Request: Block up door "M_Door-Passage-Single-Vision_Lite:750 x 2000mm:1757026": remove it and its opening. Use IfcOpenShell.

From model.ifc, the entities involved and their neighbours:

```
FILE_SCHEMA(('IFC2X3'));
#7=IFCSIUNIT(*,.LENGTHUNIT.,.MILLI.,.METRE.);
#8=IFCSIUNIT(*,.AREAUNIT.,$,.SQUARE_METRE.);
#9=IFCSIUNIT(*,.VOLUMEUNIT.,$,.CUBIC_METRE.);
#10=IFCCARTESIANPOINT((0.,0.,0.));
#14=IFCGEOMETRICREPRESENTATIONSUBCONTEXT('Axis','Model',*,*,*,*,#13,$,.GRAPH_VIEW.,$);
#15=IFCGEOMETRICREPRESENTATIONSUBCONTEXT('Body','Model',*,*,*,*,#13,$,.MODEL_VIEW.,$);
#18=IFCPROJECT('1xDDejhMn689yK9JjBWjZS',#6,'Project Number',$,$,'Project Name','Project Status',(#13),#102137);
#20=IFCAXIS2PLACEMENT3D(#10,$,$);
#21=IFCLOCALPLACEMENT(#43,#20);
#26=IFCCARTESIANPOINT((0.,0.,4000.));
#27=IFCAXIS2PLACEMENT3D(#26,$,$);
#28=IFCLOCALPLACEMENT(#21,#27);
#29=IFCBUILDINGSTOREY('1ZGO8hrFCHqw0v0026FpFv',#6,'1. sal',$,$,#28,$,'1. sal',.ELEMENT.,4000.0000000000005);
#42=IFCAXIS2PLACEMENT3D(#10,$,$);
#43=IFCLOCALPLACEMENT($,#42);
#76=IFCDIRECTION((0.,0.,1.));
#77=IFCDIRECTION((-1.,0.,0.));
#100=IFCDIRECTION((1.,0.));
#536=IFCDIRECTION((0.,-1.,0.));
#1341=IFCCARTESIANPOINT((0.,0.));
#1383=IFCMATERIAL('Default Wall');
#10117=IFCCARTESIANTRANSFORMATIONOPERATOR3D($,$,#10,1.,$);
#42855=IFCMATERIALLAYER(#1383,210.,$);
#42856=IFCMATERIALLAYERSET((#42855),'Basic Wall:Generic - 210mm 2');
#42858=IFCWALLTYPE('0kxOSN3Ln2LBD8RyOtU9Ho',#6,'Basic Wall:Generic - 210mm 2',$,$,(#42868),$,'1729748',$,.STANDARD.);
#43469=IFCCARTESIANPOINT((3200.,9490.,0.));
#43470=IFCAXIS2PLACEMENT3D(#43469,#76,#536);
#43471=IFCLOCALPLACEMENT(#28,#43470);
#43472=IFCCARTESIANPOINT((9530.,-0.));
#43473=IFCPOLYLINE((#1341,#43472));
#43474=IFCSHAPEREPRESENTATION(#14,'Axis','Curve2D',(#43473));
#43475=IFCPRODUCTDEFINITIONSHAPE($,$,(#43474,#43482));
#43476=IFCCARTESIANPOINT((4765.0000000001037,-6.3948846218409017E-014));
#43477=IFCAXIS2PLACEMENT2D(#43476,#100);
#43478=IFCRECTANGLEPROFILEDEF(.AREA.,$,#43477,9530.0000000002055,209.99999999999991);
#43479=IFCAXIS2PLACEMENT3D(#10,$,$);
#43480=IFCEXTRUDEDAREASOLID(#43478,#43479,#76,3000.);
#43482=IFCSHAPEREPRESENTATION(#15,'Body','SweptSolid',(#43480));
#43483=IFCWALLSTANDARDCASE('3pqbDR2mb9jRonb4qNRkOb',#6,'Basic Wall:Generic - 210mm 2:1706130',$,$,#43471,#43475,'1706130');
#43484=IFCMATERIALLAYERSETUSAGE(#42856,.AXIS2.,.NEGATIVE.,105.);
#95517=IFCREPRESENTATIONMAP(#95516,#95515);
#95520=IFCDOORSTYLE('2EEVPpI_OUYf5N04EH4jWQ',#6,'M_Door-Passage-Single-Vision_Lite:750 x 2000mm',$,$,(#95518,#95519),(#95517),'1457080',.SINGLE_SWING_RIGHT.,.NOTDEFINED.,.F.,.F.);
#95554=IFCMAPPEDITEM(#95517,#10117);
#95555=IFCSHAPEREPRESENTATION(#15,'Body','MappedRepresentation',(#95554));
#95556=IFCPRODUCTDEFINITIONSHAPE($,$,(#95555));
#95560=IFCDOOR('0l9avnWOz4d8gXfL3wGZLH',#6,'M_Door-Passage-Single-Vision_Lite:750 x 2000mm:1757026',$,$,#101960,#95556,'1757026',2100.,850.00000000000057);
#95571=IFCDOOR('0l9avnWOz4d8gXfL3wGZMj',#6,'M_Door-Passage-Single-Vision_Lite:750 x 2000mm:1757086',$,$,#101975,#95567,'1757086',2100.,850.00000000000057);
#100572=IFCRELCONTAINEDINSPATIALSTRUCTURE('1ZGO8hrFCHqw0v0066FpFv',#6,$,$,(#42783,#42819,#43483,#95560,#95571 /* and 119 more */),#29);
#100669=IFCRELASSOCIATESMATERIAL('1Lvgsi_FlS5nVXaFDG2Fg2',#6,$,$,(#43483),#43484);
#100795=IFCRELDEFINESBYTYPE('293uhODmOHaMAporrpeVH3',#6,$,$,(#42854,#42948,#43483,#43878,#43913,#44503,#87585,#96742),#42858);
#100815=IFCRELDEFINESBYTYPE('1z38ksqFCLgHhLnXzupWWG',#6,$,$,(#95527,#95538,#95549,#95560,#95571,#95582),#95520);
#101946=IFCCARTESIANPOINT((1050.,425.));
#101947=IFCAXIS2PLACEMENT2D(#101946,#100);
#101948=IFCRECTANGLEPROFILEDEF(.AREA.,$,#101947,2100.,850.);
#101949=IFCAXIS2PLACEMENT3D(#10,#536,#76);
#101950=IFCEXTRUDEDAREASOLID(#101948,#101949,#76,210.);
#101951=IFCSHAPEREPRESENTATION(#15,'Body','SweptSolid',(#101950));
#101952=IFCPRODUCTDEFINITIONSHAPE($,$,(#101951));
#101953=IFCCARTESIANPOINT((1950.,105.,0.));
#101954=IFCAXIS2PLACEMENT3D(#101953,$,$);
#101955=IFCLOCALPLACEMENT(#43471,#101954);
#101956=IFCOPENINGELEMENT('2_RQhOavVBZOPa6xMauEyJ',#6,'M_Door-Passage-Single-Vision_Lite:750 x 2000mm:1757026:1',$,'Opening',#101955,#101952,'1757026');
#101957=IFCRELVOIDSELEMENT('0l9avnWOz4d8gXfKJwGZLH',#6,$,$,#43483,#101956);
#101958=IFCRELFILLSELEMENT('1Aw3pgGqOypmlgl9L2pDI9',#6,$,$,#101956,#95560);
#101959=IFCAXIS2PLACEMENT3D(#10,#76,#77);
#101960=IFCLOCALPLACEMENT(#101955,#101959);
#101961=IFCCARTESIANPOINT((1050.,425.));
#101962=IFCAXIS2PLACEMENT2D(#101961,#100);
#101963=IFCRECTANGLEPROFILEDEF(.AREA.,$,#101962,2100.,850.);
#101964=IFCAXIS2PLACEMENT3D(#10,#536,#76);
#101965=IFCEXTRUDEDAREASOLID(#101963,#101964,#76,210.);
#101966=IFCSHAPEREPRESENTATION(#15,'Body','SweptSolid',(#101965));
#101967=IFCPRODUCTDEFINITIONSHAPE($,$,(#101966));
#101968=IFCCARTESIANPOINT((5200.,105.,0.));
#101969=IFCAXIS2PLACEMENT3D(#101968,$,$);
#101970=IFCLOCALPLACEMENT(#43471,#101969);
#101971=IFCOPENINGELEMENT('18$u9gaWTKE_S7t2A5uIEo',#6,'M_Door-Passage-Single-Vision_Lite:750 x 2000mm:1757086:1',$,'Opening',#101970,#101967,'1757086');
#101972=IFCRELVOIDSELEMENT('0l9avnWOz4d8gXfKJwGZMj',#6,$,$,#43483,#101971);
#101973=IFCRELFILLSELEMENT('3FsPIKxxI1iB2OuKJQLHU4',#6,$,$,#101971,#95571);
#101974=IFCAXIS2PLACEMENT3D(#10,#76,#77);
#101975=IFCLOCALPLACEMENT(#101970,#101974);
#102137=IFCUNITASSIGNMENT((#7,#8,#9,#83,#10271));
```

```python
import ifcopenshell
import ifcopenshell.api.feature
import ifcopenshell.api.root
import ifcopenshell.geom
import ifcopenshell.util.shape

model = ifcopenshell.open("model.ifc")
settings = ifcopenshell.geom.settings()


def volume(element):
    """Net volume in cubic metres, openings subtracted."""
    shape = ifcopenshell.geom.create_shape(settings, element)
    return ifcopenshell.util.shape.get_volume(shape.geometry)


door = model.by_id(95560)
opening = door.FillsVoids[0].RelatingOpeningElement
wall = opening.VoidsElements[0].RelatingBuildingElement
before = volume(wall)

ifcopenshell.api.root.remove_product(model, product=door)
ifcopenshell.api.feature.remove_feature(model, feature=opening)

after = volume(wall)

print(f"wall volume {before:.3f} -> {after:.3f} m3")

model.write("model_updated.ifc")
```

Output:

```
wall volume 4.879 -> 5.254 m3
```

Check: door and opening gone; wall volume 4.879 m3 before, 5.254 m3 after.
